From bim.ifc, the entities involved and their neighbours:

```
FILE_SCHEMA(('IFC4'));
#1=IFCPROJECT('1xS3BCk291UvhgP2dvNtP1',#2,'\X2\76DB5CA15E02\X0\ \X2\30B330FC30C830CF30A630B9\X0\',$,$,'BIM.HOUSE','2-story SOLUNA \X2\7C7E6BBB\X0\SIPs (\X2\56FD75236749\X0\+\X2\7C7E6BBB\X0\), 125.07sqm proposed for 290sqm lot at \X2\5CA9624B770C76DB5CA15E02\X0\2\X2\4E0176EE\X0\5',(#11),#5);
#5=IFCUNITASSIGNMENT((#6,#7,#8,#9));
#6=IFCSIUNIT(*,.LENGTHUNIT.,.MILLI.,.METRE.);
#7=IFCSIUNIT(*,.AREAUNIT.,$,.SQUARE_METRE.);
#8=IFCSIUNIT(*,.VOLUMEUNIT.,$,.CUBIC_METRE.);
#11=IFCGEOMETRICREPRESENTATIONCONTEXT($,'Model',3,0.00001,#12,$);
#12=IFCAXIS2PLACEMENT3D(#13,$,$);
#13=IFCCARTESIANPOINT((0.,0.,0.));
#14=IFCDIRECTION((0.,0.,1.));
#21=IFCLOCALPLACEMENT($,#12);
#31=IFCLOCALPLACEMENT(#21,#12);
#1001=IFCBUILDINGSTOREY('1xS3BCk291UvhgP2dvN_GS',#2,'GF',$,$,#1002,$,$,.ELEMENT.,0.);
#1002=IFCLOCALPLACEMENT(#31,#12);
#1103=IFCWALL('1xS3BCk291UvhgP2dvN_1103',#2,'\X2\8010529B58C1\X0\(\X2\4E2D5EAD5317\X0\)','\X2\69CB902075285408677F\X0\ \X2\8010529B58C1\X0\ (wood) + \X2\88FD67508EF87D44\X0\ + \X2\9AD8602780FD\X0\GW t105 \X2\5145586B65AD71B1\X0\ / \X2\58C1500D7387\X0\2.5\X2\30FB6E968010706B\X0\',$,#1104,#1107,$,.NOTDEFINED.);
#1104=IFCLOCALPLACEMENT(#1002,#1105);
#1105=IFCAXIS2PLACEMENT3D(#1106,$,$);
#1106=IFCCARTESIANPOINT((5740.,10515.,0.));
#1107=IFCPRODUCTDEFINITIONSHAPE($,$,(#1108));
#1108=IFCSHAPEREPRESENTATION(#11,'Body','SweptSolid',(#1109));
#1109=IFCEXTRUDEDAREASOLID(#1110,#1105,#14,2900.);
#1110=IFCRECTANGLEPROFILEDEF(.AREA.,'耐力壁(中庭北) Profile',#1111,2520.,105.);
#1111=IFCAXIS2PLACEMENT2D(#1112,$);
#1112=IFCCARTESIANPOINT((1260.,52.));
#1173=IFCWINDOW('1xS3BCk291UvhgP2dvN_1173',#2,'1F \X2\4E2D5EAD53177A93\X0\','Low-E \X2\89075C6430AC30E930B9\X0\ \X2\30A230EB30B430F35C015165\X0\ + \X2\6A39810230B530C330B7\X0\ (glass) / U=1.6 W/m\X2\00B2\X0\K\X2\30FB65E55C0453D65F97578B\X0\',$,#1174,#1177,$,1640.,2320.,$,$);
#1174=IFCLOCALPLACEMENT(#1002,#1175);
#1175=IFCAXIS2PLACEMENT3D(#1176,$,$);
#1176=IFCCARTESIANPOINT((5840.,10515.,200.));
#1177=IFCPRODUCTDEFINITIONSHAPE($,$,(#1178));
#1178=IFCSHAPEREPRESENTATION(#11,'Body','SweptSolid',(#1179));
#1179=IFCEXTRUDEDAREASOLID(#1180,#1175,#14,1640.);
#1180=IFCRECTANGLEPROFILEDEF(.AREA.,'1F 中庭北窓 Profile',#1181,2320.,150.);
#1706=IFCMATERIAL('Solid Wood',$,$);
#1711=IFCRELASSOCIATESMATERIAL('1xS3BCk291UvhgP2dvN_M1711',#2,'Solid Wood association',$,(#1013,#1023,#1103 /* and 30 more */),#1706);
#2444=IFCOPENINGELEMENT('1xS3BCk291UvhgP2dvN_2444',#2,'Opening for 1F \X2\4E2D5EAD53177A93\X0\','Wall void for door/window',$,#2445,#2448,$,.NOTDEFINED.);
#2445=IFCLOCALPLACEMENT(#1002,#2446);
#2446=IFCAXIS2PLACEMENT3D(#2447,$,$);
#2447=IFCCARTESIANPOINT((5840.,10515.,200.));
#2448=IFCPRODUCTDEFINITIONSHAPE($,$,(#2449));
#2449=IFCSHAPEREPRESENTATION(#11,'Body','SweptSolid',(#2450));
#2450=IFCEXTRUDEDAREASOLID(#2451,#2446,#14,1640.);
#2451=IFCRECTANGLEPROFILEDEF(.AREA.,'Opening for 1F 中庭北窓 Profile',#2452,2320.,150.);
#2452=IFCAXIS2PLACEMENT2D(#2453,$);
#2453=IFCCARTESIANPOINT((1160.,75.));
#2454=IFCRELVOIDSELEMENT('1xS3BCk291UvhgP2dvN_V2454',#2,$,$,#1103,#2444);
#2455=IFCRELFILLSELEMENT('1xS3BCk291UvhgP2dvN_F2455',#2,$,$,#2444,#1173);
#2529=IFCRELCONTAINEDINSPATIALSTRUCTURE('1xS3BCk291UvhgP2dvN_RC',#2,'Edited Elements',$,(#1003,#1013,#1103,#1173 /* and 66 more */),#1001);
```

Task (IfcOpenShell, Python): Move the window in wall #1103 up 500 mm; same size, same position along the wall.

```python
import numpy as np
import ifcopenshell
import ifcopenshell.api.geometry
import ifcopenshell.util.placement
import ifcopenshell.util.unit

model = ifcopenshell.open("bim.ifc")
unit_scale = ifcopenshell.util.unit.calculate_unit_scale(model)

window = model.by_id(1173)
opening = window.FillsVoids[0].RelatingOpeningElement
dz = 500.0

shift = np.array([0.0, 0.0, dz])
# The window is not placed relative to its opening, so move both.
for product in (opening, window):
    matrix = ifcopenshell.util.placement.get_local_placement(product.ObjectPlacement)
    matrix[:3, 3] += shift
    ifcopenshell.api.geometry.edit_object_placement(model, product=product, matrix=matrix, is_si=False)

print(f"moved by {dz * unit_scale:+.3f} m")

model.write("bim_updated.ifc")
```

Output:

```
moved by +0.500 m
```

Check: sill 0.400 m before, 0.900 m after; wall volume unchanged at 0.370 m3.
